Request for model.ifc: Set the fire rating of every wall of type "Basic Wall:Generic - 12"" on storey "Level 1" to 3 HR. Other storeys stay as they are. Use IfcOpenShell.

First a look at what the model holds.

```python
import ifcopenshell
import ifcopenshell.util.element

model = ifcopenshell.open("model.ifc")
print(model.schema)
storey = next(s for s in model.by_type("IfcBuildingStorey") if s.Name == "Level 1")
walls = [e for e in ifcopenshell.util.element.get_decomposition(storey) if e.is_a("IfcWall")]
seen = {}
for e in walls:
    element_type = ifcopenshell.util.element.get_type(e)
    key = (element_type.Name if element_type != e and element_type else None, ifcopenshell.util.element.get_pset(e, "Pset_WallCommon", "FireRating"))
    seen[key] = seen.get(key, 0) + 1
for (name, value), count in sorted(seen.items(), key=str):
    print(count, "x", name, "|", value)
```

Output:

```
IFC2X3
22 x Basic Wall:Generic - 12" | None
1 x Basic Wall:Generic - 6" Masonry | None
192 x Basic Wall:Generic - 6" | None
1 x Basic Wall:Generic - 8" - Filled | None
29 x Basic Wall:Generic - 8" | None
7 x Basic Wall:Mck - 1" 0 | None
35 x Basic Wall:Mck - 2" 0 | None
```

```python
import ifcopenshell
import ifcopenshell.api.pset
import ifcopenshell.util.element

model = ifcopenshell.open("model.ifc")

storey = next(s for s in model.by_type("IfcBuildingStorey") if s.Name == "Level 1")
walls = [e for e in ifcopenshell.util.element.get_decomposition(storey) if e.is_a("IfcWall")]

count = 0
for e in walls:
    element_type = ifcopenshell.util.element.get_type(e)
    if element_type in (None, e) or element_type.Name != 'Basic Wall:Generic - 12"':
        continue
    # add_pset returns the element's existing set when there is one.
    pset = ifcopenshell.api.pset.add_pset(model, product=e, name="Pset_WallCommon")
    ifcopenshell.api.pset.edit_pset(model, pset=pset, properties={"FireRating": "3 HR"})
    count += 1

print(count, "walls updated")

model.write("model_rev.ifc")
```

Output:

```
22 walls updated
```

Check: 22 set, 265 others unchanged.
